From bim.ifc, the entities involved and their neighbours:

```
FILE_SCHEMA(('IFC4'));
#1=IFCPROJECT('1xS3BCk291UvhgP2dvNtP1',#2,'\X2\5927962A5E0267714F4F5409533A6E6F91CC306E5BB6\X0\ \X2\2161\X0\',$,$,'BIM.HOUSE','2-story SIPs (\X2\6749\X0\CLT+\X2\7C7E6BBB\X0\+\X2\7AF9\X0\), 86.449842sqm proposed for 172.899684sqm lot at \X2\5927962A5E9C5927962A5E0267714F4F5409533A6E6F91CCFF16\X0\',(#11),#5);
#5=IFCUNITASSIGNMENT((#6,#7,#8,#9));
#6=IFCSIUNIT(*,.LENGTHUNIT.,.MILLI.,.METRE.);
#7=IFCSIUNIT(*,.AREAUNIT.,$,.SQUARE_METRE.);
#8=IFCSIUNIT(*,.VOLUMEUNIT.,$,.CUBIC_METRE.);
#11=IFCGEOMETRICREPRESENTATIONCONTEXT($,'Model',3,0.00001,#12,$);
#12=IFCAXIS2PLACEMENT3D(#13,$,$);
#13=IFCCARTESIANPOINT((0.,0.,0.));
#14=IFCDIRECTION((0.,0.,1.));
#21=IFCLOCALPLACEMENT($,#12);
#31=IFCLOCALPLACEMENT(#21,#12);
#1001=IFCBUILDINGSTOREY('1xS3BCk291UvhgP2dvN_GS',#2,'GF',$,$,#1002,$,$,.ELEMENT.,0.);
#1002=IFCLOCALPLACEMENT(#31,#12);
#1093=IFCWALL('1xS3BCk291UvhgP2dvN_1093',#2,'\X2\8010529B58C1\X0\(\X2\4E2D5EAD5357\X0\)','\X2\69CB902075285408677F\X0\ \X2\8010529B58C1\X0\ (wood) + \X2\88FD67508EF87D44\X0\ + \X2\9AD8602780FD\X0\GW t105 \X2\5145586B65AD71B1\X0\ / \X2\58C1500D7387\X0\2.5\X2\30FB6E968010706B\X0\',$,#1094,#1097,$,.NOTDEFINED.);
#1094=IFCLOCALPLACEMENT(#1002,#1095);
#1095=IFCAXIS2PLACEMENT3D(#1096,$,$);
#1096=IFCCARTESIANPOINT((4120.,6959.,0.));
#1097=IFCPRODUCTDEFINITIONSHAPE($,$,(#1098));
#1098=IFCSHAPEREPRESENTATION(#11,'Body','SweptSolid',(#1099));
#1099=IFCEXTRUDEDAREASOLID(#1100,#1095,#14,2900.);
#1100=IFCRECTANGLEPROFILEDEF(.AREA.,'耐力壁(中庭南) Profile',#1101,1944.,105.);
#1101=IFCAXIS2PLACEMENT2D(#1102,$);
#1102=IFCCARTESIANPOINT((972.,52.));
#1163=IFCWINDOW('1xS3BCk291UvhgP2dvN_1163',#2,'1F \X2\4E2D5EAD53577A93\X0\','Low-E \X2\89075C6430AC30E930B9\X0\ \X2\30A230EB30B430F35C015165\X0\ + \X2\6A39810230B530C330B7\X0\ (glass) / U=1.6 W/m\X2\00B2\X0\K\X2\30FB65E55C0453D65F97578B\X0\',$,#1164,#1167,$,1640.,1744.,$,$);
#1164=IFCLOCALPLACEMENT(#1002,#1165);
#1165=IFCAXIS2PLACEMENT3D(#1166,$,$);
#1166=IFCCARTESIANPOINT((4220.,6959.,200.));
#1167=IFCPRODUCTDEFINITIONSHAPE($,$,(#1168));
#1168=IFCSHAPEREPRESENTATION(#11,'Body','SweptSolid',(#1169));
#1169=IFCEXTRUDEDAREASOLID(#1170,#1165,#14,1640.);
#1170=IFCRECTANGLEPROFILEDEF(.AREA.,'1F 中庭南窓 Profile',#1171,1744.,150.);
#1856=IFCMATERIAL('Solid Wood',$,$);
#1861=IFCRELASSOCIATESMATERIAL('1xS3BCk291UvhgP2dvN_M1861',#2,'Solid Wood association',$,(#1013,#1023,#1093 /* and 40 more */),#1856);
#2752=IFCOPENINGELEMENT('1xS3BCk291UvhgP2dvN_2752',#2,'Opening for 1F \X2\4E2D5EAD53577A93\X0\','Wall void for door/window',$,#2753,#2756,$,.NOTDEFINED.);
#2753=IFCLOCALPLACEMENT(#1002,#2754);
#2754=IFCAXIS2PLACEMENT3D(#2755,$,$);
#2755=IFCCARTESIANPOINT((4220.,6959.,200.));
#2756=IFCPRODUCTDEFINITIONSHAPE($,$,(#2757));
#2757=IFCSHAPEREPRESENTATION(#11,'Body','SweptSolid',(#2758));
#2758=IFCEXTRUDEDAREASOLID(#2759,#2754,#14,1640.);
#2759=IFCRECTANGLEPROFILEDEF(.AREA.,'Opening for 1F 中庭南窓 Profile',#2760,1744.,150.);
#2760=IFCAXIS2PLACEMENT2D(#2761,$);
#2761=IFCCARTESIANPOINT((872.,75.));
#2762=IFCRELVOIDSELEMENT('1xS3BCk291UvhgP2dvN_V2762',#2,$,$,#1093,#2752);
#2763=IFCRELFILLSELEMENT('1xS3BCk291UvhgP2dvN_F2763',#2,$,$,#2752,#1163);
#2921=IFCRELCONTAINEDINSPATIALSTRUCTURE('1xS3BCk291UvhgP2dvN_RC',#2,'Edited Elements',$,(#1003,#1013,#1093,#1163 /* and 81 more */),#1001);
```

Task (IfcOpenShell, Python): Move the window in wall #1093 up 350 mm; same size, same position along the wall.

```python
import numpy as np
import ifcopenshell
import ifcopenshell.api.geometry
import ifcopenshell.util.placement
import ifcopenshell.util.unit

model = ifcopenshell.open("bim.ifc")
unit_scale = ifcopenshell.util.unit.calculate_unit_scale(model)

window = model.by_guid("1xS3BCk291UvhgP2dvN_1163")
opening = window.FillsVoids[0].RelatingOpeningElement
dz = 350.0

shift = np.array([0.0, 0.0, dz])
# The window is not placed relative to its opening, so move both.
for product in (opening, window):
    matrix = ifcopenshell.util.placement.get_local_placement(product.ObjectPlacement)
    matrix[:3, 3] += shift
    ifcopenshell.api.geometry.edit_object_placement(model, product=product, matrix=matrix, is_si=False)

print(f"moved by {dz * unit_scale:+.3f} m")

model.write("bim_rev.ifc")
```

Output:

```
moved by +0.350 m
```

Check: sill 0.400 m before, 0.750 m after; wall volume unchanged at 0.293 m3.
